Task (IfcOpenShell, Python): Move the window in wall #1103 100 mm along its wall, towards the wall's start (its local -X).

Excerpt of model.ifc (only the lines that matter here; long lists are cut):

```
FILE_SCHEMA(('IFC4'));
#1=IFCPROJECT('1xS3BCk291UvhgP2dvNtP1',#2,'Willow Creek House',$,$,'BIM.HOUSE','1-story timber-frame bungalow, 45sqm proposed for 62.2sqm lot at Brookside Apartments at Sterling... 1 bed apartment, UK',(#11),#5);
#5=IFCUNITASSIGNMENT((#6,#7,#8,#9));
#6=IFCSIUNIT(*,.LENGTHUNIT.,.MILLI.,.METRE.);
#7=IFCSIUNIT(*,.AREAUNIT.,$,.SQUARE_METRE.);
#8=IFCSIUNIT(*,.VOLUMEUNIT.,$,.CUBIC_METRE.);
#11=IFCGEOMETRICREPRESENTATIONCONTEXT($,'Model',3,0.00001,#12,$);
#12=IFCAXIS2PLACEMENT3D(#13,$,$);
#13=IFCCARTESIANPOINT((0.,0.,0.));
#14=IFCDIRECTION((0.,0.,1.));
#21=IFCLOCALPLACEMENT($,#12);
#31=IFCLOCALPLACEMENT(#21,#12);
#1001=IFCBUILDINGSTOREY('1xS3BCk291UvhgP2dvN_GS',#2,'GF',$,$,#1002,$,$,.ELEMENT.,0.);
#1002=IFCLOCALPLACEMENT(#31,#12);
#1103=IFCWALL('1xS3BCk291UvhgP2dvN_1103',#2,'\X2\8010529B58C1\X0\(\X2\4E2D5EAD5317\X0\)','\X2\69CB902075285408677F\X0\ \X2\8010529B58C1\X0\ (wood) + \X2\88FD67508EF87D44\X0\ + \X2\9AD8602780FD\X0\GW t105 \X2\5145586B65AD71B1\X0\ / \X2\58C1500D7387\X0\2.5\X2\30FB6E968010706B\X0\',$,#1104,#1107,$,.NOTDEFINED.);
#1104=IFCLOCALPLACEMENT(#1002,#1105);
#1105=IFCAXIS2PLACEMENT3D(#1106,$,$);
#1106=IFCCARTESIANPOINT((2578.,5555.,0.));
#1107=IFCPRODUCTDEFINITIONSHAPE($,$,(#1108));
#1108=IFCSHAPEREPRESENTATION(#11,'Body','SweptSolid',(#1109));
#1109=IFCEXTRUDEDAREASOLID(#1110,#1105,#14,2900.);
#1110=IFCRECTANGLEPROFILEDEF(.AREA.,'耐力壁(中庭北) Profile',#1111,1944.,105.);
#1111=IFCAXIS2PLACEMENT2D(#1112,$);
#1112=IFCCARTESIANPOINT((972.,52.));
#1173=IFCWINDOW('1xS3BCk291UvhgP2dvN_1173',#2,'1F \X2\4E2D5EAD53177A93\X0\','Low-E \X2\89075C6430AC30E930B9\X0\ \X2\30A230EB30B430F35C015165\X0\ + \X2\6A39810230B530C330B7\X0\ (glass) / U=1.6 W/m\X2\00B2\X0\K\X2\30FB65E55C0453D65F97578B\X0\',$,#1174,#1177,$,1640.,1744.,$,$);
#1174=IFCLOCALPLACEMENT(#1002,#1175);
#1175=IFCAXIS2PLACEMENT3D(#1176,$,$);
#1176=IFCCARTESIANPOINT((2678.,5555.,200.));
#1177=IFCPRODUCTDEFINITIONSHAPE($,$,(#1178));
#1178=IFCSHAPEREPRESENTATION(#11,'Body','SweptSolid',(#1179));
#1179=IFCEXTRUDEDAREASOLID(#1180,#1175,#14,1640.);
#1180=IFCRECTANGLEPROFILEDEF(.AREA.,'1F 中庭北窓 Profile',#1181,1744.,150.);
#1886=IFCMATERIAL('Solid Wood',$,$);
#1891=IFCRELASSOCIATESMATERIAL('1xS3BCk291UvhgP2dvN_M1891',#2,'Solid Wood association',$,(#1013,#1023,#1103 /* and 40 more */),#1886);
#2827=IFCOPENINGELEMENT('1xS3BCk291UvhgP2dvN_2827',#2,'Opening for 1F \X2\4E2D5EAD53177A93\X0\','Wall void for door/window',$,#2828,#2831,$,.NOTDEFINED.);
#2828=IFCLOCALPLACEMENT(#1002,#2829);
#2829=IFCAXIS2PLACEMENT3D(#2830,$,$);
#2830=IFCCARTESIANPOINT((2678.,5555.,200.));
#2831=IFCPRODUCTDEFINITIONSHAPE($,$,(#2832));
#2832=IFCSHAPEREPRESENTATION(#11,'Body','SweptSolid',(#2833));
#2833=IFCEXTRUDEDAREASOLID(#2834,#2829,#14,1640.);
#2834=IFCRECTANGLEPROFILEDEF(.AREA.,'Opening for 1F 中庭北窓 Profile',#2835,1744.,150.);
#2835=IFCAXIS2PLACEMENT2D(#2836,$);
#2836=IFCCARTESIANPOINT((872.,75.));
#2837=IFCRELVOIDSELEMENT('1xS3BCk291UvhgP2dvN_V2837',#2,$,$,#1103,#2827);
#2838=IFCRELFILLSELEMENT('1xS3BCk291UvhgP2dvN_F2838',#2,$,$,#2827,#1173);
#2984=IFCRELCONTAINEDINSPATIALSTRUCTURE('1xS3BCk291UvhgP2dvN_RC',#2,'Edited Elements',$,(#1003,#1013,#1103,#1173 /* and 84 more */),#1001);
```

```python
import ifcopenshell
import ifcopenshell.api.geometry
import ifcopenshell.util.placement

model = ifcopenshell.open("model.ifc")

window = model.by_guid("1xS3BCk291UvhgP2dvN_1173")
opening = window.FillsVoids[0].RelatingOpeningElement
wall = opening.VoidsElements[0].RelatingBuildingElement

wall_matrix = ifcopenshell.util.placement.get_local_placement(wall.ObjectPlacement)
shift = wall_matrix[:3, 0] * -100.0
before = ifcopenshell.util.placement.get_local_placement(window.ObjectPlacement)[:3, 3].copy()

# The window is not placed relative to its opening, so move both.
for product in (opening, window):
    matrix = ifcopenshell.util.placement.get_local_placement(product.ObjectPlacement)
    matrix[:3, 3] += shift
    ifcopenshell.api.geometry.edit_object_placement(model, product=product, matrix=matrix, is_si=False)

after = ifcopenshell.util.placement.get_local_placement(window.ObjectPlacement)[:3, 3]
print("window moved by", (after - before).round(3) + 0.0)

model.write("model_rev.ifc")
```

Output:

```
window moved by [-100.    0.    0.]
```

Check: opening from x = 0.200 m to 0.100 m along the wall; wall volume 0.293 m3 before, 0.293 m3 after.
